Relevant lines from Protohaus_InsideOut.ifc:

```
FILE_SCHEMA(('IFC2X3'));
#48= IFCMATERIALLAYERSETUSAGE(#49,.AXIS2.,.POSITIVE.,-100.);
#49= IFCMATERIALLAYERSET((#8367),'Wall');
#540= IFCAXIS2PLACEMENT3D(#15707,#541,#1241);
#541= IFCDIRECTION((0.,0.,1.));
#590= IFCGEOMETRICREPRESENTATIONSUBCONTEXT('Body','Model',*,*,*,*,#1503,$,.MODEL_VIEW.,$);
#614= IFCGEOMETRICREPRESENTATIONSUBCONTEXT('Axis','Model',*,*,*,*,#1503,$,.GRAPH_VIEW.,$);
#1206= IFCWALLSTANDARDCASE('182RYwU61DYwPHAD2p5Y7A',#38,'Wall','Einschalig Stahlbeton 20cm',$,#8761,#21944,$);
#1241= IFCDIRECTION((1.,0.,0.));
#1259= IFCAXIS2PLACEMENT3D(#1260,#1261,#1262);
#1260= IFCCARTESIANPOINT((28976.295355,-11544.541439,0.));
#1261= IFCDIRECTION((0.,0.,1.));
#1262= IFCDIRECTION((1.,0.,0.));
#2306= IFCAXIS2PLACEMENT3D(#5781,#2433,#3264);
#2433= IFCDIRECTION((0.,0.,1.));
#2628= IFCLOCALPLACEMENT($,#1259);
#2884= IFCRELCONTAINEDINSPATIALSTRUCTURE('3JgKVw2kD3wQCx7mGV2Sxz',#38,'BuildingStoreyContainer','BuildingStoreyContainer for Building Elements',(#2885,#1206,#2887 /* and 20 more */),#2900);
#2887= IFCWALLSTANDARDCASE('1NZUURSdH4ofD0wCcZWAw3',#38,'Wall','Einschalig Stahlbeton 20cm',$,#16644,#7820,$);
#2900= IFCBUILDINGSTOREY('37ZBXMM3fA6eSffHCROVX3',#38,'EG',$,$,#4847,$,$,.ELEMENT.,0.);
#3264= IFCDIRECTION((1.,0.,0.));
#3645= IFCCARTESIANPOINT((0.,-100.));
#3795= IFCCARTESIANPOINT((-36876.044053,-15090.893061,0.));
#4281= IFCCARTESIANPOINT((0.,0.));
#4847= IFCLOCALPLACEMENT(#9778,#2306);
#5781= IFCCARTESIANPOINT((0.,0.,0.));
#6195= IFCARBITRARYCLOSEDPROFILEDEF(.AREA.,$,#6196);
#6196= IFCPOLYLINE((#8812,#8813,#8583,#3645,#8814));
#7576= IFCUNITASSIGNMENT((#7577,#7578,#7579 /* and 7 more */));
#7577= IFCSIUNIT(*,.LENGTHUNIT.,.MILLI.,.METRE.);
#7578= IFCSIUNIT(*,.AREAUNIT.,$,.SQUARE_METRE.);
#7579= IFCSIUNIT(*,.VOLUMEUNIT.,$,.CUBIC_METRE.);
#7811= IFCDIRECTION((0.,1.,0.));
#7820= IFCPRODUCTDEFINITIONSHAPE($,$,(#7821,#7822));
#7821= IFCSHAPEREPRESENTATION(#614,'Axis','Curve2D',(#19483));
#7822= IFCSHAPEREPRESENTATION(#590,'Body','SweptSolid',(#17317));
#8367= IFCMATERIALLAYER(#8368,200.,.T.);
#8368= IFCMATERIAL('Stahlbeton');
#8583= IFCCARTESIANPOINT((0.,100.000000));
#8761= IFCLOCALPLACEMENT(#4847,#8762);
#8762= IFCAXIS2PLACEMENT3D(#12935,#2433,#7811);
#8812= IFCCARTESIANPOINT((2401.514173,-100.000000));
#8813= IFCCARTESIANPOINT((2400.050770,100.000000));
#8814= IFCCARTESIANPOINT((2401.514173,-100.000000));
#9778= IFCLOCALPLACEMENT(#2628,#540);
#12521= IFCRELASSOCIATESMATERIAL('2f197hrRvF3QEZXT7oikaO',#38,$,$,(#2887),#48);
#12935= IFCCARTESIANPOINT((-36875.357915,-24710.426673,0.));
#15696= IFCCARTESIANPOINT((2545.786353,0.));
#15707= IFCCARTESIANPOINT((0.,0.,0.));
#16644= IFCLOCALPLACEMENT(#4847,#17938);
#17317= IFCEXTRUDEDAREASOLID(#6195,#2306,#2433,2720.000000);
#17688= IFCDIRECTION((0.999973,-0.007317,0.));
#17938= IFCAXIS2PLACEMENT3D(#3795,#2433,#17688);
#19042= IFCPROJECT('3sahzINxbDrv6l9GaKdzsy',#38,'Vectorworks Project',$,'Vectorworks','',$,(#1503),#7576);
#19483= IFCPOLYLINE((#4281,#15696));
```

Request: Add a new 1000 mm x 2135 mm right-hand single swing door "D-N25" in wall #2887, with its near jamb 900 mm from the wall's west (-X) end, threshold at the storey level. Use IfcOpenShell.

```python
import numpy as np
import ifcopenshell
import ifcopenshell.api.feature
import ifcopenshell.api.geometry
import ifcopenshell.api.root
import ifcopenshell.api.spatial
import ifcopenshell.api.type
import ifcopenshell.geom
import ifcopenshell.util.element
import ifcopenshell.util.placement
import ifcopenshell.util.representation
import ifcopenshell.util.shape
import ifcopenshell.util.unit

model = ifcopenshell.open("Protohaus_InsideOut.ifc")
unit_scale = ifcopenshell.util.unit.calculate_unit_scale(model)
settings = ifcopenshell.geom.settings()


def volume(element):
    """Net volume in cubic metres, openings subtracted."""
    shape = ifcopenshell.geom.create_shape(settings, element)
    return ifcopenshell.util.shape.get_volume(shape.geometry)


wall = model.by_id(2887)
storey = ifcopenshell.util.element.get_container(wall, ifc_class="IfcBuildingStorey")
context = ifcopenshell.util.representation.get_context(model, "Model", "Body", "MODEL_VIEW")
before = volume(wall)

width, height, from_end, sill = 1, 2.135, 0.9, 0.0  # metres

# The wall runs along its own X axis, and the end named is its -X end.
wall_shape = ifcopenshell.geom.create_shape(settings, wall)
x, y, z = ifcopenshell.util.shape.get_vertices(wall_shape.geometry).T
start = x.min() + from_end
face, thickness = float(y.min()), float(y.max() - y.min())
wall_matrix = ifcopenshell.util.placement.get_local_placement(wall.ObjectPlacement)
level = ifcopenshell.util.placement.get_local_placement(storey.ObjectPlacement)[2, 3]


def in_wall(x, y):
    """Placement at x, y metres in the wall's axes, at sill height."""
    matrix = wall_matrix.copy()
    matrix[:, 3] = wall_matrix @ np.array([x / unit_scale, y / unit_scale, 0.0, 1.0])
    matrix[2, 3] = level + sill / unit_scale
    return matrix


# Opening: a box that overshoots both wall faces by 50 mm.
opening = ifcopenshell.api.root.create_entity(model, ifc_class="IfcOpeningElement")
box = ifcopenshell.api.geometry.add_wall_representation(
    model, context=context, length=width, height=height, thickness=thickness + 0.1
)
ifcopenshell.api.geometry.assign_representation(model, product=opening, representation=box)
ifcopenshell.api.geometry.edit_object_placement(model, product=opening, matrix=in_wall(start, face - 0.05), is_si=False)
ifcopenshell.api.feature.add_feature(model, feature=opening, element=wall)

door = ifcopenshell.api.root.create_entity(model, ifc_class="IfcDoor", name="D-N25")
door.OverallWidth, door.OverallHeight = width / unit_scale, height / unit_scale
body = ifcopenshell.api.geometry.add_door_representation(
    model,
    context=context,
    overall_width=door.OverallWidth,
    overall_height=door.OverallHeight,
    operation_type="SINGLE_SWING_RIGHT",
    lining_properties={"LiningDepth": thickness / unit_scale, "ThresholdDepth": thickness / unit_scale},
)
ifcopenshell.api.geometry.assign_representation(model, product=door, representation=body)
ifcopenshell.api.spatial.assign_container(model, products=[door], relating_structure=storey)
fills = ifcopenshell.api.feature.add_filling(model, opening=opening, element=door)
fills.OwnerHistory = door.OwnerHistory  # required in IFC2X3

# IFC2X3 keeps the operation on the door style.
style = ifcopenshell.api.root.create_entity(model, ifc_class="IfcDoorStyle", name="D-N25")
style.OperationType, style.ConstructionType = "SINGLE_SWING_RIGHT", "NOTDEFINED"
style.ParameterTakesPrecedence = style.Sizeable = False
ifcopenshell.api.type.assign_type(model, related_objects=[door], relating_type=style)

# The lining spans the wall, so the door starts at the wall face.
ifcopenshell.api.geometry.edit_object_placement(model, product=door, matrix=in_wall(start, face), is_si=False)

after = volume(wall)

print(f"wall volume {before:.3f} -> {after:.3f} m3")

model.write("Protohaus_InsideOut_edited.ifc")
```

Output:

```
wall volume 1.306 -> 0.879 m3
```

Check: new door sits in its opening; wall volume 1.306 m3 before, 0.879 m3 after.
